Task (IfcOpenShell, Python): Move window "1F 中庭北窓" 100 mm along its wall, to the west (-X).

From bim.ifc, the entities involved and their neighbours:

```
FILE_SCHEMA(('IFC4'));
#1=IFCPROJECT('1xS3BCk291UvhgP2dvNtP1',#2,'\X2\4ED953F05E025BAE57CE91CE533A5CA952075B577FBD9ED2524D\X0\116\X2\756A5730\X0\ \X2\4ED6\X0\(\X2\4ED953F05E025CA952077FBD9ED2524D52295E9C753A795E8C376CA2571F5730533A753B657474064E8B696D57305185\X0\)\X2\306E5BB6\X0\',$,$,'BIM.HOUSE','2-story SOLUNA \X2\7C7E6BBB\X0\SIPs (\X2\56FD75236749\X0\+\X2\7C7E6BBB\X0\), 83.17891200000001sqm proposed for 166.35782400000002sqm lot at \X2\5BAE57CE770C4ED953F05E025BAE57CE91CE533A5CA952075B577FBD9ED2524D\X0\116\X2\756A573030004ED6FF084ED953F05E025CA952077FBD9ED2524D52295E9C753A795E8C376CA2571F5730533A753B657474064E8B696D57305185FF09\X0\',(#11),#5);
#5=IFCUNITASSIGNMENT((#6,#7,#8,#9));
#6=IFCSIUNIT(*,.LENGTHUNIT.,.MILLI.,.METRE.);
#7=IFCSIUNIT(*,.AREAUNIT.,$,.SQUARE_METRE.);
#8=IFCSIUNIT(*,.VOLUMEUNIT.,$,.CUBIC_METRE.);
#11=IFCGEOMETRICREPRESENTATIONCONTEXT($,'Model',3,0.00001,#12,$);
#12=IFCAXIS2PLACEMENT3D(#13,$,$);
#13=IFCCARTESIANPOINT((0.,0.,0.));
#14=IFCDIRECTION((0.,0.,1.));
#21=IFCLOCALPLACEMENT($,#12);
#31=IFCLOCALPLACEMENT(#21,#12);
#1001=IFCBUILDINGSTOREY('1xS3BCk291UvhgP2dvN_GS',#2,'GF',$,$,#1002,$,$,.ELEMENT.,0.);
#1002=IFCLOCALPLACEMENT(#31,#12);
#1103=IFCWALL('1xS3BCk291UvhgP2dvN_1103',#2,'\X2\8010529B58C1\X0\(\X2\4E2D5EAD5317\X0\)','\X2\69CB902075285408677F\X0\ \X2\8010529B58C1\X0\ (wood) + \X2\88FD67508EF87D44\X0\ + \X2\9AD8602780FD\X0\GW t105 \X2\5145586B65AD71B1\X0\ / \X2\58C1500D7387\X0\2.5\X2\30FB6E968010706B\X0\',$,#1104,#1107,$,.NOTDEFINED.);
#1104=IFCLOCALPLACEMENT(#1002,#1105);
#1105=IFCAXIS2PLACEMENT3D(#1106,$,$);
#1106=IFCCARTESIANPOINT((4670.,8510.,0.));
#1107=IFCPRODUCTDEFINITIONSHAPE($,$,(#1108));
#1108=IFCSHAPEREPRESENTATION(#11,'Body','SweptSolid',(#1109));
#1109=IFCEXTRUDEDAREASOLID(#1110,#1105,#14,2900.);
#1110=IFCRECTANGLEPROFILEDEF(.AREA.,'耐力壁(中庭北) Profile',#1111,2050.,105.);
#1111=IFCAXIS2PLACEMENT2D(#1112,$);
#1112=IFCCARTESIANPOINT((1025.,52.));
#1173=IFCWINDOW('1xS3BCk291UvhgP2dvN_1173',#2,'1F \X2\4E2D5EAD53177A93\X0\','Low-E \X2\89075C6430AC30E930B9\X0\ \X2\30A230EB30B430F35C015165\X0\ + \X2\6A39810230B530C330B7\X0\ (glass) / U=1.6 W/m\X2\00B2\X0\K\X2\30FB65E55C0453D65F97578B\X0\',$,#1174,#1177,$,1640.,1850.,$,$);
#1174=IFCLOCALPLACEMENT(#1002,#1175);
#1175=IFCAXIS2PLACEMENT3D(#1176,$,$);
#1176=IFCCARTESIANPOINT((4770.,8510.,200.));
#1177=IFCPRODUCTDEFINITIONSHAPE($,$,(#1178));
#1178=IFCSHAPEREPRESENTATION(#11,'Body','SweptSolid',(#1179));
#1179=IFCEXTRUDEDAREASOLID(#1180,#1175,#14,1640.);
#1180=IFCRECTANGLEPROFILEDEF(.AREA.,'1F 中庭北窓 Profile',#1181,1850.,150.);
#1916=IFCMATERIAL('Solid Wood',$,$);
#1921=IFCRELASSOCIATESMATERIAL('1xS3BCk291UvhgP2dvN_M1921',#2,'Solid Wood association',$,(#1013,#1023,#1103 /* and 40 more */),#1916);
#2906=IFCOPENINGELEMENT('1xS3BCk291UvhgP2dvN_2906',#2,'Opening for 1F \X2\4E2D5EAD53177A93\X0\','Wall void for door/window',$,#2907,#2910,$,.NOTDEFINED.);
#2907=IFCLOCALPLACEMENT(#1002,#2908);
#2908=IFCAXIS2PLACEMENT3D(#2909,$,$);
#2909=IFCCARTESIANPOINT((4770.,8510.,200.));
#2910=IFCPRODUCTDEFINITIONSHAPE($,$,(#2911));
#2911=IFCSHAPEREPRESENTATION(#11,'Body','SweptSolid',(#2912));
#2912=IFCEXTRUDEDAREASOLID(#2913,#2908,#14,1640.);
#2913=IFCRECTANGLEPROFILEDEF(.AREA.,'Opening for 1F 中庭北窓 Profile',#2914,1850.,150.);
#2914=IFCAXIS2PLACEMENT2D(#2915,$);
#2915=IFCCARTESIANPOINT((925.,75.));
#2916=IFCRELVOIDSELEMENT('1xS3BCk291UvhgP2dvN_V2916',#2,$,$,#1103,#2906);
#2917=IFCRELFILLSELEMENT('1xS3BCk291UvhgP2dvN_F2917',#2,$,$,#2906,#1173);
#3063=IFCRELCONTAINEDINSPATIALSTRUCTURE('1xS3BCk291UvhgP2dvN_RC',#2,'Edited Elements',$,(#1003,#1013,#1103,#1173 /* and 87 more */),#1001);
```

```python
import ifcopenshell
import ifcopenshell.api.geometry
import ifcopenshell.util.placement

model = ifcopenshell.open("bim.ifc")

window = model.by_guid("1xS3BCk291UvhgP2dvN_1173")
opening = window.FillsVoids[0].RelatingOpeningElement
wall = opening.VoidsElements[0].RelatingBuildingElement

wall_matrix = ifcopenshell.util.placement.get_local_placement(wall.ObjectPlacement)
shift = wall_matrix[:3, 0] * -100.0
before = ifcopenshell.util.placement.get_local_placement(window.ObjectPlacement)[:3, 3].copy()

# The window is not placed relative to its opening, so move both.
for product in (opening, window):
    matrix = ifcopenshell.util.placement.get_local_placement(product.ObjectPlacement)
    matrix[:3, 3] += shift
    ifcopenshell.api.geometry.edit_object_placement(model, product=product, matrix=matrix, is_si=False)

after = ifcopenshell.util.placement.get_local_placement(window.ObjectPlacement)[:3, 3]
print("window moved by", (after - before).round(3) + 0.0)

model.write("bim_v2.ifc")
```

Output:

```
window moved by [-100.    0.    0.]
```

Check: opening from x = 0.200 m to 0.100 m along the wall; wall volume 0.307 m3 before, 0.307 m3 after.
